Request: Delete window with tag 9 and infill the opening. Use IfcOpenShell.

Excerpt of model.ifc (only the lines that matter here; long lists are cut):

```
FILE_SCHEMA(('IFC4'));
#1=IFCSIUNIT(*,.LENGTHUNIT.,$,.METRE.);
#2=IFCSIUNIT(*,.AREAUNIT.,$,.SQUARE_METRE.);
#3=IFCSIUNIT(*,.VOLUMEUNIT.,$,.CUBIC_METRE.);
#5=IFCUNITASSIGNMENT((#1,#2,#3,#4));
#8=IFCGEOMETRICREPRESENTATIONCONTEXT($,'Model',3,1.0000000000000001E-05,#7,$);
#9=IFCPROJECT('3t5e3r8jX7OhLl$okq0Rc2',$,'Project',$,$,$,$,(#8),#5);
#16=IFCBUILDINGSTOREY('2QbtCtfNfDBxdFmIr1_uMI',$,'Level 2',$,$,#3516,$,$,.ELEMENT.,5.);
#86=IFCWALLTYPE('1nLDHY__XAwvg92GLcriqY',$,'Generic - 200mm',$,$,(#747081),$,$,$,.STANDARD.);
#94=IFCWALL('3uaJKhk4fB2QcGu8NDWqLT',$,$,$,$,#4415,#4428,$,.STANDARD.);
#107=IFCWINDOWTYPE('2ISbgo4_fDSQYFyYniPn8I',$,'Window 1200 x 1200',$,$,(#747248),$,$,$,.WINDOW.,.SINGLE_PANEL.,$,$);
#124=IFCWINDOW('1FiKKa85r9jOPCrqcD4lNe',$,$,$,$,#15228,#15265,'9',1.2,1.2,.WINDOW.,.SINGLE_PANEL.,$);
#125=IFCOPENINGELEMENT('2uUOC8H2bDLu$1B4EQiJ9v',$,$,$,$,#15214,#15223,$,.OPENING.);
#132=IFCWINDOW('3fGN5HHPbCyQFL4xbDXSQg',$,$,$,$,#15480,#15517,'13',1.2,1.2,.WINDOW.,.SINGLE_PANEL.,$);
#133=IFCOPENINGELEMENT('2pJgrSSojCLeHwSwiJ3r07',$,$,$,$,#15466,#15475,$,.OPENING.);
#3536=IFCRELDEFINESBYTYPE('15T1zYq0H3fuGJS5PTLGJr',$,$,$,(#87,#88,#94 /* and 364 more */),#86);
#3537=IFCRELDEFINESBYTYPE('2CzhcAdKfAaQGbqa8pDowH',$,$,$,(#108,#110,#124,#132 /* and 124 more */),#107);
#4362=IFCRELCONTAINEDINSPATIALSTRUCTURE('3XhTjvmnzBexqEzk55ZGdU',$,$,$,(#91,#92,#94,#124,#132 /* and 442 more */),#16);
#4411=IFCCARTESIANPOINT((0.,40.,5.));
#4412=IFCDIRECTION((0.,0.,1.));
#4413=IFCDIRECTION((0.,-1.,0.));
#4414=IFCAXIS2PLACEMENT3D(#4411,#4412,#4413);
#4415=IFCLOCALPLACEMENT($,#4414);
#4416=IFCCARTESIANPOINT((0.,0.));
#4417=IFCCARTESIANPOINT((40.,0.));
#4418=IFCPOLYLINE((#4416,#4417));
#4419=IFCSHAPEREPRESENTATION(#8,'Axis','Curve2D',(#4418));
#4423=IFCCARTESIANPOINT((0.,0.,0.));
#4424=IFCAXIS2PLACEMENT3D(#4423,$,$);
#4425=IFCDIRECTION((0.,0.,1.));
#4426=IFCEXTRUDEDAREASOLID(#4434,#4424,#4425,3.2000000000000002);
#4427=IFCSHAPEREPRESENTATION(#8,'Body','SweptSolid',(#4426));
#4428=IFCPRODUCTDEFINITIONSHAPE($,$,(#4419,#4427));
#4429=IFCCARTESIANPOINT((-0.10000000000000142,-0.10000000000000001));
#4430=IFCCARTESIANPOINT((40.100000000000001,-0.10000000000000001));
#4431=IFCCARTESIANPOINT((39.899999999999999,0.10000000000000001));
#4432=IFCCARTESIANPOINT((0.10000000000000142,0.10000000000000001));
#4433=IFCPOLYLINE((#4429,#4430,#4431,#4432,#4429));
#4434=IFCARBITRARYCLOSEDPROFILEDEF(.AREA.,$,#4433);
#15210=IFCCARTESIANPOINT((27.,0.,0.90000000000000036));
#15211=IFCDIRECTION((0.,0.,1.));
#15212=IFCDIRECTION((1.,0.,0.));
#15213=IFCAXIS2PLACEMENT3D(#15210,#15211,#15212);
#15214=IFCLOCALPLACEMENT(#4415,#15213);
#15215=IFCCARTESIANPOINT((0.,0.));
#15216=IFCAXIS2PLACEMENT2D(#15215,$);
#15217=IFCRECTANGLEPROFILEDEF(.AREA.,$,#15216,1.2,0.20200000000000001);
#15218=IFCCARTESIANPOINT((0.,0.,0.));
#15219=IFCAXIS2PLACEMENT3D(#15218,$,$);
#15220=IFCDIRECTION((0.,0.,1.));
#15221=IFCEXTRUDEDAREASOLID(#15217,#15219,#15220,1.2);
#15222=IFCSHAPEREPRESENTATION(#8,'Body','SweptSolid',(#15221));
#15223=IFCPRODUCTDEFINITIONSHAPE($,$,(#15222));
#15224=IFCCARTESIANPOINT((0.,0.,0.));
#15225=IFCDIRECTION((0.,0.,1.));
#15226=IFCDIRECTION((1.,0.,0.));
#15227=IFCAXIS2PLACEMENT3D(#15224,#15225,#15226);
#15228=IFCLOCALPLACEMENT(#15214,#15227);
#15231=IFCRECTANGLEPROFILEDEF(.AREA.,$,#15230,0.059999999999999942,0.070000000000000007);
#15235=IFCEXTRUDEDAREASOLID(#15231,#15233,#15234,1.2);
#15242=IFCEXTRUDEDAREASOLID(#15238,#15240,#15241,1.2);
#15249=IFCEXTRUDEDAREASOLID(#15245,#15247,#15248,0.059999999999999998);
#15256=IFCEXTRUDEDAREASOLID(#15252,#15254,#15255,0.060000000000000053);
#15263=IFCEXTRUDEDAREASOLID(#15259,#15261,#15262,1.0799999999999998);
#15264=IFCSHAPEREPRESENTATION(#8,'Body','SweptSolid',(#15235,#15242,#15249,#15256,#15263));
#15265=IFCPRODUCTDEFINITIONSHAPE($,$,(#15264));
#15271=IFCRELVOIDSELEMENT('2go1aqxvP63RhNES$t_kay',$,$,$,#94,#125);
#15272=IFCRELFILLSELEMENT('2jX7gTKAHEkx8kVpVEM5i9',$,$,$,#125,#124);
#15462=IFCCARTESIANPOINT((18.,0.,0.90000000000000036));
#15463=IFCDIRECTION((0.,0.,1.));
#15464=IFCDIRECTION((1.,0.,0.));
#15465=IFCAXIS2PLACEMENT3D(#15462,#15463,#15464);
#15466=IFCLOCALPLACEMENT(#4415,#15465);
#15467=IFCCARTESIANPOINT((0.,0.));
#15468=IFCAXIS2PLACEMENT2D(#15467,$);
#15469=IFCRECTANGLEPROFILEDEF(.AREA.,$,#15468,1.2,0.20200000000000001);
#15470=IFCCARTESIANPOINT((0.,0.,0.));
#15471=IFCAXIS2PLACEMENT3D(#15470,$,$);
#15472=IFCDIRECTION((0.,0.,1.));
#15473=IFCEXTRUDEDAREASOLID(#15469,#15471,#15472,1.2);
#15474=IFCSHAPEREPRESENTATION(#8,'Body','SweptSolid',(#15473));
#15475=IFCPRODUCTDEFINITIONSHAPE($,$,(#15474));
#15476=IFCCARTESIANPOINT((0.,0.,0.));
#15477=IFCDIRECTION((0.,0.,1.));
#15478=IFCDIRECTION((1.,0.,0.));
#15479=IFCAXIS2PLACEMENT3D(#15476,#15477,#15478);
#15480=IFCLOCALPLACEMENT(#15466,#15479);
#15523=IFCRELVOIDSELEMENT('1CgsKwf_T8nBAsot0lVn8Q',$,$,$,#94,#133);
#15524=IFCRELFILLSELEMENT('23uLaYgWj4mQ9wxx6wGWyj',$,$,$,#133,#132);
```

```python
import ifcopenshell
import ifcopenshell.api.feature
import ifcopenshell.api.root
import ifcopenshell.geom
import ifcopenshell.util.shape

model = ifcopenshell.open("model.ifc")
settings = ifcopenshell.geom.settings()


def volume(element):
    """Net volume in cubic metres, openings subtracted."""
    shape = ifcopenshell.geom.create_shape(settings, element)
    return ifcopenshell.util.shape.get_volume(shape.geometry)


window = model.by_guid("1FiKKa85r9jOPCrqcD4lNe")
opening = window.FillsVoids[0].RelatingOpeningElement
wall = opening.VoidsElements[0].RelatingBuildingElement
before = volume(wall)

ifcopenshell.api.root.remove_product(model, product=window)
ifcopenshell.api.feature.remove_feature(model, feature=opening)

after = volume(wall)

print(f"wall volume {before:.3f} -> {after:.3f} m3")

model.write("model-out.ifc")
```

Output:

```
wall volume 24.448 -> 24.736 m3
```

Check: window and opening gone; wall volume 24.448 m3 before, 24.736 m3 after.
